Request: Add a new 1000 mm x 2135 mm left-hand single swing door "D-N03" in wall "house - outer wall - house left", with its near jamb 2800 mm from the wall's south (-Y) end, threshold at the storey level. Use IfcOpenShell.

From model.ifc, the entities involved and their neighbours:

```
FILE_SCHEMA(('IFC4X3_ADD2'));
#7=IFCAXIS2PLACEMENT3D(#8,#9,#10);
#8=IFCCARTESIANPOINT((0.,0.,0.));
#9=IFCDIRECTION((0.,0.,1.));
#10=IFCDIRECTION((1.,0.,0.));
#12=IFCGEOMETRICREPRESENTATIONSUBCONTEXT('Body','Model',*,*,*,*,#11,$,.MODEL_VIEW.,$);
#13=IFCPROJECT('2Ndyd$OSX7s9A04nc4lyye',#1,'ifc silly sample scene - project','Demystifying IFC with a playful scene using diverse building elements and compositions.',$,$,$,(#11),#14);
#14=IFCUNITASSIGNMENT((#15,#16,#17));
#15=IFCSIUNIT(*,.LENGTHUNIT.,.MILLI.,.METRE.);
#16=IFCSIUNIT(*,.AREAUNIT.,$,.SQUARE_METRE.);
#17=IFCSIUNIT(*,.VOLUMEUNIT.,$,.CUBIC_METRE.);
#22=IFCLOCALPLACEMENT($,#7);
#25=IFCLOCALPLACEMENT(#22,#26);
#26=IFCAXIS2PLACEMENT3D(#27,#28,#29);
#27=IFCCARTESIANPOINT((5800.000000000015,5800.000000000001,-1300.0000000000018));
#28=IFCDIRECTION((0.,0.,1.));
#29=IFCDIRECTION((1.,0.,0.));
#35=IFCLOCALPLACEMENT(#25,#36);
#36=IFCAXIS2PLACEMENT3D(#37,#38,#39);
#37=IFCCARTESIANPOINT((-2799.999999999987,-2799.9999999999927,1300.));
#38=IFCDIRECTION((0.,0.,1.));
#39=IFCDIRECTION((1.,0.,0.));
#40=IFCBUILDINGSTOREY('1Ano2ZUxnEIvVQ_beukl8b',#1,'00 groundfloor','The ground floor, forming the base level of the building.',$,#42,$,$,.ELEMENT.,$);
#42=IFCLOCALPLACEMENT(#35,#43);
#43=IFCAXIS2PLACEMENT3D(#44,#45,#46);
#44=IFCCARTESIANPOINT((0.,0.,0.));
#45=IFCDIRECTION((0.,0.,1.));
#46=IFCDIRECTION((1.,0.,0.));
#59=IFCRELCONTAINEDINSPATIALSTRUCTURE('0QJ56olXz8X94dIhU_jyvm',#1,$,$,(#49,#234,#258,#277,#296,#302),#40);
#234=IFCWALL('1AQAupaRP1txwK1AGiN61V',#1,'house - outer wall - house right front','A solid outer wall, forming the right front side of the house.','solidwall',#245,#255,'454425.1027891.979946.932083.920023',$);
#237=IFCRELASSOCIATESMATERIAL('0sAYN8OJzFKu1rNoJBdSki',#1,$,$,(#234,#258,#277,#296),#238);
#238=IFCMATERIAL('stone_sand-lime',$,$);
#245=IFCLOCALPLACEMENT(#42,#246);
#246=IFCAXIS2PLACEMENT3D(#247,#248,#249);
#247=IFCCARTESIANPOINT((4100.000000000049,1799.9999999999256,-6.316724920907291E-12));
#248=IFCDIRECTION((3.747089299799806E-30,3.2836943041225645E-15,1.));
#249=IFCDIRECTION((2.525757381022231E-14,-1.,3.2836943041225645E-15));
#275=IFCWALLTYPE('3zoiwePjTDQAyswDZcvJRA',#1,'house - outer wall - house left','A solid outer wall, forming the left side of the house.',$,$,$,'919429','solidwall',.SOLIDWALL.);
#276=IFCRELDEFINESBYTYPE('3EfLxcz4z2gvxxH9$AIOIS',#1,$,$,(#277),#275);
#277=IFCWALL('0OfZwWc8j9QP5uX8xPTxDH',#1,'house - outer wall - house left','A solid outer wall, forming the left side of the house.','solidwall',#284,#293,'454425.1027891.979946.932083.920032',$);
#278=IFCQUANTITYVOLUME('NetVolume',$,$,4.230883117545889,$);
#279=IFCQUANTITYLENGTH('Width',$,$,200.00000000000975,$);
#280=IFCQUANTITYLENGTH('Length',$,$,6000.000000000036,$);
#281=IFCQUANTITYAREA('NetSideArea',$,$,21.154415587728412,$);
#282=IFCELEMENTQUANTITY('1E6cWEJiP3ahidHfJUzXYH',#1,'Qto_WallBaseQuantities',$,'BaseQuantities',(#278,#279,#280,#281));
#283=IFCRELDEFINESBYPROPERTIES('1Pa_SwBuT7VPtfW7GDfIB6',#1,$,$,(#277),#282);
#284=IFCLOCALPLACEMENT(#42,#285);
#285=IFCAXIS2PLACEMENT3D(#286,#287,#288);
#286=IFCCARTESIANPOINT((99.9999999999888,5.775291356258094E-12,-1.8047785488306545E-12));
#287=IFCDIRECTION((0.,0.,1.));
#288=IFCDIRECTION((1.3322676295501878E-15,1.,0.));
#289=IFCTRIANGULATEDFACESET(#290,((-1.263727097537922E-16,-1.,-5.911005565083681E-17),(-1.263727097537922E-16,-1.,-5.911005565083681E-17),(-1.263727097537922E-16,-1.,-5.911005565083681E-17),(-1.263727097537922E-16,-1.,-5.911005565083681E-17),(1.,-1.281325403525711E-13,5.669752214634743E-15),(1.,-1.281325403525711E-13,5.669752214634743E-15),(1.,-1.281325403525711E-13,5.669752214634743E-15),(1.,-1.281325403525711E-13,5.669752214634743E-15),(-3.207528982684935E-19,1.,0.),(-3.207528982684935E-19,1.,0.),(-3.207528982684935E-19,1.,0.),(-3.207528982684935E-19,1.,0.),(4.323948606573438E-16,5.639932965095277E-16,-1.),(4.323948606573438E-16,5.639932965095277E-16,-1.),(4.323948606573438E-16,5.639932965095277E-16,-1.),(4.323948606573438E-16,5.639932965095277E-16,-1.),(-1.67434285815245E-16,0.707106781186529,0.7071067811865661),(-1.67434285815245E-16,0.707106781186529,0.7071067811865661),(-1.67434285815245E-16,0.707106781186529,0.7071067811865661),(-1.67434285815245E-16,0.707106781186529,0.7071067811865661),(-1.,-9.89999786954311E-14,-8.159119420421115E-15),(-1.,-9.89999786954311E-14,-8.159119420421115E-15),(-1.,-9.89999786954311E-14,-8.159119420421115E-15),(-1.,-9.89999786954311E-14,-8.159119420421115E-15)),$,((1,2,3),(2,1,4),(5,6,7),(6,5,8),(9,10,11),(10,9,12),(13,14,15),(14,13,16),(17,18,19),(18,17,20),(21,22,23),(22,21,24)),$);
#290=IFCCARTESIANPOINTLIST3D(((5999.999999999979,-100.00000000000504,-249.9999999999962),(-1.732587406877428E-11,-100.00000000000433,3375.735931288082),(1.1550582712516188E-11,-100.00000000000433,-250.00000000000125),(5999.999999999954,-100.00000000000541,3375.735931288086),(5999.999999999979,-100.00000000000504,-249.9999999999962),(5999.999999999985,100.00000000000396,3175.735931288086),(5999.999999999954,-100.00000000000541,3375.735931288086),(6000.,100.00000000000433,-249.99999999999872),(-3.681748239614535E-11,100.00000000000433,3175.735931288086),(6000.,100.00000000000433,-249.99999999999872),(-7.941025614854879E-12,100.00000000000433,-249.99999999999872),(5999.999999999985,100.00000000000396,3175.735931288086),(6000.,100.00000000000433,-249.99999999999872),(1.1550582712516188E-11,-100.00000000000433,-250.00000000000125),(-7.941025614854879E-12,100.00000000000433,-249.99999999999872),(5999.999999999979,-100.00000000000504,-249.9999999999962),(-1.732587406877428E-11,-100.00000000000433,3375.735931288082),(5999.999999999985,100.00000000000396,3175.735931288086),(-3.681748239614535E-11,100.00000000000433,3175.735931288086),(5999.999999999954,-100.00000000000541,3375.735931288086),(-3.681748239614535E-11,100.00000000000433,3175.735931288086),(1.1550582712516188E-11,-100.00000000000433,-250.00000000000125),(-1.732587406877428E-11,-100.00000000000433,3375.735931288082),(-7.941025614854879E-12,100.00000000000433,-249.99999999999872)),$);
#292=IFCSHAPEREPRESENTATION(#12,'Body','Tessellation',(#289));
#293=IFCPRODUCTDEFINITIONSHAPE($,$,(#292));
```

```python
import numpy as np
import ifcopenshell
import ifcopenshell.api.feature
import ifcopenshell.api.geometry
import ifcopenshell.api.pset
import ifcopenshell.api.root
import ifcopenshell.api.spatial
import ifcopenshell.geom
import ifcopenshell.util.element
import ifcopenshell.util.placement
import ifcopenshell.util.representation
import ifcopenshell.util.shape
import ifcopenshell.util.unit

model = ifcopenshell.open("model.ifc")
unit_scale = ifcopenshell.util.unit.calculate_unit_scale(model)
area_scale = ifcopenshell.util.unit.calculate_unit_scale(model, "AREAUNIT")
volume_scale = ifcopenshell.util.unit.calculate_unit_scale(model, "VOLUMEUNIT")
settings = ifcopenshell.geom.settings()


def volume(element):
    """Net volume in cubic metres, openings subtracted."""
    shape = ifcopenshell.geom.create_shape(settings, element)
    return ifcopenshell.util.shape.get_volume(shape.geometry)


wall = model.by_guid("0OfZwWc8j9QP5uX8xPTxDH")
storey = ifcopenshell.util.element.get_container(wall, ifc_class="IfcBuildingStorey")
context = ifcopenshell.util.representation.get_context(model, "Model", "Body", "MODEL_VIEW")
before = volume(wall)

width, height, from_end, sill = 1, 2.135, 2.8, 0.0  # metres

# The wall runs along its own X axis, and the end named is its -X end.
wall_shape = ifcopenshell.geom.create_shape(settings, wall)
x, y, z = ifcopenshell.util.shape.get_vertices(wall_shape.geometry).T
start = x.min() + from_end
face, thickness = float(y.min()), float(y.max() - y.min())
wall_matrix = ifcopenshell.util.placement.get_local_placement(wall.ObjectPlacement)
level = ifcopenshell.util.placement.get_local_placement(storey.ObjectPlacement)[2, 3]


def in_wall(x, y):
    """Placement at x, y metres in the wall's axes, at sill height."""
    matrix = wall_matrix.copy()
    matrix[:, 3] = wall_matrix @ np.array([x / unit_scale, y / unit_scale, 0.0, 1.0])
    matrix[2, 3] = level + sill / unit_scale
    return matrix


# Opening: a box that overshoots both wall faces by 50 mm.
opening = ifcopenshell.api.root.create_entity(model, ifc_class="IfcOpeningElement", predefined_type="OPENING")
box = ifcopenshell.api.geometry.add_wall_representation(
    model, context=context, length=width, height=height, thickness=thickness + 0.1
)
ifcopenshell.api.geometry.assign_representation(model, product=opening, representation=box)
ifcopenshell.api.geometry.edit_object_placement(model, product=opening, matrix=in_wall(start, face - 0.05), is_si=False)
ifcopenshell.api.feature.add_feature(model, feature=opening, element=wall)

door = ifcopenshell.api.root.create_entity(model, ifc_class="IfcDoor", name="D-N03", predefined_type="DOOR")
door.OverallWidth, door.OverallHeight = width / unit_scale, height / unit_scale
door.OperationType = "SINGLE_SWING_LEFT"
body = ifcopenshell.api.geometry.add_door_representation(
    model,
    context=context,
    overall_width=door.OverallWidth,
    overall_height=door.OverallHeight,
    operation_type="SINGLE_SWING_LEFT",
    lining_properties={"LiningDepth": thickness / unit_scale, "ThresholdDepth": thickness / unit_scale},
)
ifcopenshell.api.geometry.assign_representation(model, product=door, representation=body)
ifcopenshell.api.spatial.assign_container(model, products=[door], relating_structure=storey)
ifcopenshell.api.feature.add_filling(model, opening=opening, element=door)

# The lining spans the wall, so the door starts at the wall face.
ifcopenshell.api.geometry.edit_object_placement(model, product=door, matrix=in_wall(start, face), is_si=False)

after = volume(wall)

# Update the wall's stored quantities.
qto = model.by_id(ifcopenshell.util.element.get_pset(wall, "Qto_WallBaseQuantities", should_inherit=False)["id"])
ifcopenshell.api.pset.edit_qto(model, qto=qto, properties={
    "NetVolume": after / volume_scale,
    "NetSideArea": after / thickness / area_scale,
})

print(f"wall volume {before:.3f} -> {after:.3f} m3")

model.write("model_updated.ifc")
```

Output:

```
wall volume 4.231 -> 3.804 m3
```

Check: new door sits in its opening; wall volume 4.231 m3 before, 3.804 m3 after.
